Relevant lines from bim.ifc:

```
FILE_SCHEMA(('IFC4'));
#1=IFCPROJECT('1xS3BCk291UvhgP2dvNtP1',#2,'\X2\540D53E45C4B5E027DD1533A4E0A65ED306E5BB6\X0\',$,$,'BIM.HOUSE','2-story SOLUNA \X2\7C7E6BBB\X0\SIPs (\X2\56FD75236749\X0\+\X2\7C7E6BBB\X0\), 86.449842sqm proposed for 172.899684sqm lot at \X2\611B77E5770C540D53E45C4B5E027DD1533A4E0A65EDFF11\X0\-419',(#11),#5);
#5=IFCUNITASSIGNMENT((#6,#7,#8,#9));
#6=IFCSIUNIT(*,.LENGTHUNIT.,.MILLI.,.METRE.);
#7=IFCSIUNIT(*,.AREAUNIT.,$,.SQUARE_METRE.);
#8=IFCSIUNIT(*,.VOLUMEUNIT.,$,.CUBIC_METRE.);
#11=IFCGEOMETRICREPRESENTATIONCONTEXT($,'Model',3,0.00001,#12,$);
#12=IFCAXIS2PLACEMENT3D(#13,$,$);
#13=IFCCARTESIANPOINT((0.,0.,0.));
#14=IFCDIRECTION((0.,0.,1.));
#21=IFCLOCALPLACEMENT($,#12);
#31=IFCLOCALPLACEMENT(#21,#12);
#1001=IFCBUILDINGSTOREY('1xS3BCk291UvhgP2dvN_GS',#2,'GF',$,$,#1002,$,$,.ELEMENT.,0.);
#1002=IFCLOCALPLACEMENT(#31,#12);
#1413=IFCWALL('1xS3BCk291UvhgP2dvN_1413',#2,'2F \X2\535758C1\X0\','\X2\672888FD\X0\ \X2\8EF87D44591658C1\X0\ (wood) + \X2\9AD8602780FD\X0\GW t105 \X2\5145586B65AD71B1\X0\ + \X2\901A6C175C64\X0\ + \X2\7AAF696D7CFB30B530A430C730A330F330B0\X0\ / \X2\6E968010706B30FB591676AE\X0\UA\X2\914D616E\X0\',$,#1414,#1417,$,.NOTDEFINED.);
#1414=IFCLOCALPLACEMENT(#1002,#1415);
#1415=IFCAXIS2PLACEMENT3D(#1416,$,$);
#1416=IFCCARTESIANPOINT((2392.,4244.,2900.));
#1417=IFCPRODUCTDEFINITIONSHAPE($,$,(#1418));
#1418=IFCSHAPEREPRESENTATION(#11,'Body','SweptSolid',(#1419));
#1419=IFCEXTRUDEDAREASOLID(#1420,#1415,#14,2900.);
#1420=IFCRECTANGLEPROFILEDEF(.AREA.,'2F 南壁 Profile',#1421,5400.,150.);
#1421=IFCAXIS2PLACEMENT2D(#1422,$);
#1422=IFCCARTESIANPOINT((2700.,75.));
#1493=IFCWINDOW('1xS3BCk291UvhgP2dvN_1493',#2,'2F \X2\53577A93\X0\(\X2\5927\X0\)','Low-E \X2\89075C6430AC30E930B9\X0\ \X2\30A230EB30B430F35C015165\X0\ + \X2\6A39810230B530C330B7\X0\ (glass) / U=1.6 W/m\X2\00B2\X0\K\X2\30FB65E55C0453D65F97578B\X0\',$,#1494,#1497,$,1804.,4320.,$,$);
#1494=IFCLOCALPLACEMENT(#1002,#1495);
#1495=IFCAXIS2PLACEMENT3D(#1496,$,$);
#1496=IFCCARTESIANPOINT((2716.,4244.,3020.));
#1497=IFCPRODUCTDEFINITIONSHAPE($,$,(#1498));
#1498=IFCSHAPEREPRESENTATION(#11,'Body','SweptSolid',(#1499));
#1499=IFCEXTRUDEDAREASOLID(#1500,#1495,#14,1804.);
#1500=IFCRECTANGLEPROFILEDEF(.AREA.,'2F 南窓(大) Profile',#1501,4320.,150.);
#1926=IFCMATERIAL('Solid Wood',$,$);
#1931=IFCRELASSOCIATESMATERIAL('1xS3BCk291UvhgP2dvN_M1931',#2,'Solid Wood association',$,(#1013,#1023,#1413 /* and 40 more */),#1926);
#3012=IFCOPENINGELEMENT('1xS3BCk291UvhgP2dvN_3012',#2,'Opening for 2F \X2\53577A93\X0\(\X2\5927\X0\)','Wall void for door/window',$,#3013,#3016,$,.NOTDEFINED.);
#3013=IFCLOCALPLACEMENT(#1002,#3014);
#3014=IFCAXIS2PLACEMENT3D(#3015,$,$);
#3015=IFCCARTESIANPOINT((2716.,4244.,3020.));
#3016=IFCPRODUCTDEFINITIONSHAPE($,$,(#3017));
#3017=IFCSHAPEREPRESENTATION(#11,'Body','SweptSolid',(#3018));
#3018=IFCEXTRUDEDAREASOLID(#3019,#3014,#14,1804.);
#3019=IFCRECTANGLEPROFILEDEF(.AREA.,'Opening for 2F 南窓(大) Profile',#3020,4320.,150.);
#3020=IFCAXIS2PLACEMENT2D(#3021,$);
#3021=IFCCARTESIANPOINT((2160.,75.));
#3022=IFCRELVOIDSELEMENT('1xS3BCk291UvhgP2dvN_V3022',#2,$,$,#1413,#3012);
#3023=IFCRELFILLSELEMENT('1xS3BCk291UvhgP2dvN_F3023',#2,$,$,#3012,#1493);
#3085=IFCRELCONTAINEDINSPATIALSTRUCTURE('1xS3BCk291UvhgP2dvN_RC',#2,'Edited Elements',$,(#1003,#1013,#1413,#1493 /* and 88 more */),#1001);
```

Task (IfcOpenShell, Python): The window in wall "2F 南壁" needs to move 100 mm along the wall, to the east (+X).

```python
import ifcopenshell
import ifcopenshell.api.geometry
import ifcopenshell.util.placement
import ifcopenshell.util.unit

model = ifcopenshell.open("bim.ifc")
unit_scale = ifcopenshell.util.unit.calculate_unit_scale(model)

window = model.by_guid("1xS3BCk291UvhgP2dvN_1493")
opening = window.FillsVoids[0].RelatingOpeningElement
wall = opening.VoidsElements[0].RelatingBuildingElement

wall_matrix = ifcopenshell.util.placement.get_local_placement(wall.ObjectPlacement)
shift = wall_matrix[:3, 0] * 0.1 / unit_scale
before = ifcopenshell.util.placement.get_local_placement(window.ObjectPlacement)[:3, 3].copy()

# The window is not placed relative to its opening, so move both.
for product in (opening, window):
    matrix = ifcopenshell.util.placement.get_local_placement(product.ObjectPlacement)
    matrix[:3, 3] += shift
    ifcopenshell.api.geometry.edit_object_placement(model, product=product, matrix=matrix, is_si=False)

after = ifcopenshell.util.placement.get_local_placement(window.ObjectPlacement)[:3, 3]
print("window moved by", (after - before).round(3) + 0.0)

model.write("bim_v2.ifc")
```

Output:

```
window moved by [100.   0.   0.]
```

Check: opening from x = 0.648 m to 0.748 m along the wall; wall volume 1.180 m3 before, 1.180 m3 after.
